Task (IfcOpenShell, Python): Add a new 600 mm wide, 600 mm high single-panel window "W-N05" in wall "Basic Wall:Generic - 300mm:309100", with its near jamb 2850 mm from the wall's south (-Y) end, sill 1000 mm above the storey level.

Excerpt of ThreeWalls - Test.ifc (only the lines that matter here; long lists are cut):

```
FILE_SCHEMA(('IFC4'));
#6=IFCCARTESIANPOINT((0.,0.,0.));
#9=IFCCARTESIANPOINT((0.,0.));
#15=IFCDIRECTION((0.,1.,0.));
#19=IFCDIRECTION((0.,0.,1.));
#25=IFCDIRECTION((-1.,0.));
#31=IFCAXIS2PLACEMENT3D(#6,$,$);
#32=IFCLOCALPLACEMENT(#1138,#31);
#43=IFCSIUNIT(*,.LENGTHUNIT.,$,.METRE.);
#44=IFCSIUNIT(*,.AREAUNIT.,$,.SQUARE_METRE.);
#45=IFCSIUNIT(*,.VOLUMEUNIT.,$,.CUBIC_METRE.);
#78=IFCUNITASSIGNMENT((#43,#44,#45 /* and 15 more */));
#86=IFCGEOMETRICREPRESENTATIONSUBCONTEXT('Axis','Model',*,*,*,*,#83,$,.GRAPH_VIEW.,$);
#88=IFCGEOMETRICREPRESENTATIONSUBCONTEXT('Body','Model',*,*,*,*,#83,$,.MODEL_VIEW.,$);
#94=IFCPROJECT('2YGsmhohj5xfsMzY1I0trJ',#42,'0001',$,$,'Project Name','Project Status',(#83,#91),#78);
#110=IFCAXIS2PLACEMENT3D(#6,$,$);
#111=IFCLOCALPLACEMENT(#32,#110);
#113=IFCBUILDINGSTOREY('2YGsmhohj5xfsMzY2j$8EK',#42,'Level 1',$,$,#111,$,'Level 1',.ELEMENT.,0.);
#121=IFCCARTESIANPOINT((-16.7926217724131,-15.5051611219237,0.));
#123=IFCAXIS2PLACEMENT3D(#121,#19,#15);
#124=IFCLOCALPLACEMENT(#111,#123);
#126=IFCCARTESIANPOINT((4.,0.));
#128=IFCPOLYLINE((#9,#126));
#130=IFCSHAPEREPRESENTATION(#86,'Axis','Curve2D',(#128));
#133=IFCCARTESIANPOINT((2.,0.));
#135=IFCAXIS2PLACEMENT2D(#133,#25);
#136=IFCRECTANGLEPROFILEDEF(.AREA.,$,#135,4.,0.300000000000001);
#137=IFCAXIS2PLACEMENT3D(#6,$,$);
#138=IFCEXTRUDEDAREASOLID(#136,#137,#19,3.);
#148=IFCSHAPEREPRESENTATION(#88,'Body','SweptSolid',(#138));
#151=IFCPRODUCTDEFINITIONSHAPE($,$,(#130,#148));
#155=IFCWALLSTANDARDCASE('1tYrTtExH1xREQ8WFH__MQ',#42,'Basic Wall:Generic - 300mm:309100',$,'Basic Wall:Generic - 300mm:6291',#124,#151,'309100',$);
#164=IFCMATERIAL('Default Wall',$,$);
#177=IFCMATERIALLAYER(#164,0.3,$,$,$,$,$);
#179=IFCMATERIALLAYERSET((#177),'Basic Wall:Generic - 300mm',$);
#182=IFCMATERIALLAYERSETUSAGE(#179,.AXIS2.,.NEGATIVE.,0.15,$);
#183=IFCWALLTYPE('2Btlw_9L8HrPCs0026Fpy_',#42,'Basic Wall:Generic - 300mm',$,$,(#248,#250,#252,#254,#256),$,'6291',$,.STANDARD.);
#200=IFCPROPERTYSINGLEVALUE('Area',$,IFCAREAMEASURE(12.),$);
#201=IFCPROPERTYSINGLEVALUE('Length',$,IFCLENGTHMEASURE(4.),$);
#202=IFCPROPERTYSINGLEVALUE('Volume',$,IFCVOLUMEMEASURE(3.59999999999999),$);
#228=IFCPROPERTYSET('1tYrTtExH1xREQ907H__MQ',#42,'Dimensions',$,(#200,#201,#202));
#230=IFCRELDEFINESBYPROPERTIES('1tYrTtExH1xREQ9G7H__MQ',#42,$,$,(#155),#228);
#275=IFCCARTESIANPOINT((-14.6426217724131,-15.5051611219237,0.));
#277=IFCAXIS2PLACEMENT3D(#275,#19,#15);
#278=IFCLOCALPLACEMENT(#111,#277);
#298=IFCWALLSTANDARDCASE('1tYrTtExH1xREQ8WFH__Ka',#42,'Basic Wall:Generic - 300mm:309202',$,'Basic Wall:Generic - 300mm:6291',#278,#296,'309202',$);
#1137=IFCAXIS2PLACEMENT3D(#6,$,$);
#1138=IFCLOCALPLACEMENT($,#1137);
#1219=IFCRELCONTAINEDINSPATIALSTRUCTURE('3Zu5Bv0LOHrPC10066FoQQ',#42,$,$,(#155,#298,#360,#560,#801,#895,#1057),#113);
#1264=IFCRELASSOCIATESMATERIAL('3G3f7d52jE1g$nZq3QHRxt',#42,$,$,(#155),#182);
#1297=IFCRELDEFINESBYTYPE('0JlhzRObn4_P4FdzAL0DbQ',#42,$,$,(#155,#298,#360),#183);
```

```python
import numpy as np
import ifcopenshell
import ifcopenshell.api.feature
import ifcopenshell.api.geometry
import ifcopenshell.api.pset
import ifcopenshell.api.root
import ifcopenshell.api.spatial
import ifcopenshell.geom
import ifcopenshell.util.element
import ifcopenshell.util.placement
import ifcopenshell.util.representation
import ifcopenshell.util.shape
import ifcopenshell.util.unit

model = ifcopenshell.open("ThreeWalls - Test.ifc")
unit_scale = ifcopenshell.util.unit.calculate_unit_scale(model)
area_scale = ifcopenshell.util.unit.calculate_unit_scale(model, "AREAUNIT")
volume_scale = ifcopenshell.util.unit.calculate_unit_scale(model, "VOLUMEUNIT")
settings = ifcopenshell.geom.settings()


def volume(element):
    """Net volume in cubic metres, openings subtracted."""
    shape = ifcopenshell.geom.create_shape(settings, element)
    return ifcopenshell.util.shape.get_volume(shape.geometry)


wall = model.by_guid("1tYrTtExH1xREQ8WFH__MQ")
storey = ifcopenshell.util.element.get_container(wall, ifc_class="IfcBuildingStorey")
context = ifcopenshell.util.representation.get_context(model, "Model", "Body", "MODEL_VIEW")
before = volume(wall)

width, height, from_end, sill = 0.6, 0.6, 2.85, 1  # metres

# The wall runs along its own X axis, and the end named is its -X end.
wall_shape = ifcopenshell.geom.create_shape(settings, wall)
x, y, z = ifcopenshell.util.shape.get_vertices(wall_shape.geometry).T
start = x.min() + from_end
face, thickness = float(y.min()), float(y.max() - y.min())
wall_matrix = ifcopenshell.util.placement.get_local_placement(wall.ObjectPlacement)
level = ifcopenshell.util.placement.get_local_placement(storey.ObjectPlacement)[2, 3]


def in_wall(x, y):
    """Placement at x, y metres in the wall's axes, at sill height."""
    matrix = wall_matrix.copy()
    matrix[:, 3] = wall_matrix @ np.array([x / unit_scale, y / unit_scale, 0.0, 1.0])
    matrix[2, 3] = level + sill / unit_scale
    return matrix


# Opening: a box that overshoots both wall faces by 50 mm.
opening = ifcopenshell.api.root.create_entity(model, ifc_class="IfcOpeningElement", predefined_type="OPENING")
box = ifcopenshell.api.geometry.add_wall_representation(
    model, context=context, length=width, height=height, thickness=thickness + 0.1
)
ifcopenshell.api.geometry.assign_representation(model, product=opening, representation=box)
ifcopenshell.api.geometry.edit_object_placement(model, product=opening, matrix=in_wall(start, face - 0.05), is_si=False)
ifcopenshell.api.feature.add_feature(model, feature=opening, element=wall)

window = ifcopenshell.api.root.create_entity(model, ifc_class="IfcWindow", name="W-N05", predefined_type="WINDOW")
window.OverallWidth, window.OverallHeight = width / unit_scale, height / unit_scale
window.PartitioningType = "SINGLE_PANEL"
body = ifcopenshell.api.geometry.add_window_representation(
    model,
    context=context,
    overall_width=window.OverallWidth,
    overall_height=window.OverallHeight,
    partition_type="SINGLE_PANEL",
)
ifcopenshell.api.geometry.assign_representation(model, product=window, representation=body)
ifcopenshell.api.spatial.assign_container(model, products=[window], relating_structure=storey)
ifcopenshell.api.feature.add_filling(model, opening=opening, element=window)

# Centre the window in the wall's thickness.
ifcopenshell.api.geometry.edit_object_placement(model, product=window, matrix=in_wall(start, face), is_si=False)
window_shape = ifcopenshell.geom.create_shape(settings, window)
depth = ifcopenshell.util.shape.get_vertices(window_shape.geometry)[:, 1]
offset = face + thickness / 2 - (depth.min() + depth.max()) / 2
ifcopenshell.api.geometry.edit_object_placement(model, product=window, matrix=in_wall(start, offset), is_si=False)

after = volume(wall)

# Update the wall's stored quantities.
pset = model.by_id(ifcopenshell.util.element.get_pset(wall, "Dimensions", should_inherit=False)["id"])
ifcopenshell.api.pset.edit_pset(model, pset=pset, properties={
    "Area": model.create_entity("IfcAreaMeasure", after / thickness / area_scale),
    "Volume": model.create_entity("IfcVolumeMeasure", after / volume_scale),
})

print(f"wall volume {before:.3f} -> {after:.3f} m3")

model.write("ThreeWalls - Test_v2.ifc")
```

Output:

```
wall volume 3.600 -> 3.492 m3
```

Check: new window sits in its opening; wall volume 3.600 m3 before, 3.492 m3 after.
